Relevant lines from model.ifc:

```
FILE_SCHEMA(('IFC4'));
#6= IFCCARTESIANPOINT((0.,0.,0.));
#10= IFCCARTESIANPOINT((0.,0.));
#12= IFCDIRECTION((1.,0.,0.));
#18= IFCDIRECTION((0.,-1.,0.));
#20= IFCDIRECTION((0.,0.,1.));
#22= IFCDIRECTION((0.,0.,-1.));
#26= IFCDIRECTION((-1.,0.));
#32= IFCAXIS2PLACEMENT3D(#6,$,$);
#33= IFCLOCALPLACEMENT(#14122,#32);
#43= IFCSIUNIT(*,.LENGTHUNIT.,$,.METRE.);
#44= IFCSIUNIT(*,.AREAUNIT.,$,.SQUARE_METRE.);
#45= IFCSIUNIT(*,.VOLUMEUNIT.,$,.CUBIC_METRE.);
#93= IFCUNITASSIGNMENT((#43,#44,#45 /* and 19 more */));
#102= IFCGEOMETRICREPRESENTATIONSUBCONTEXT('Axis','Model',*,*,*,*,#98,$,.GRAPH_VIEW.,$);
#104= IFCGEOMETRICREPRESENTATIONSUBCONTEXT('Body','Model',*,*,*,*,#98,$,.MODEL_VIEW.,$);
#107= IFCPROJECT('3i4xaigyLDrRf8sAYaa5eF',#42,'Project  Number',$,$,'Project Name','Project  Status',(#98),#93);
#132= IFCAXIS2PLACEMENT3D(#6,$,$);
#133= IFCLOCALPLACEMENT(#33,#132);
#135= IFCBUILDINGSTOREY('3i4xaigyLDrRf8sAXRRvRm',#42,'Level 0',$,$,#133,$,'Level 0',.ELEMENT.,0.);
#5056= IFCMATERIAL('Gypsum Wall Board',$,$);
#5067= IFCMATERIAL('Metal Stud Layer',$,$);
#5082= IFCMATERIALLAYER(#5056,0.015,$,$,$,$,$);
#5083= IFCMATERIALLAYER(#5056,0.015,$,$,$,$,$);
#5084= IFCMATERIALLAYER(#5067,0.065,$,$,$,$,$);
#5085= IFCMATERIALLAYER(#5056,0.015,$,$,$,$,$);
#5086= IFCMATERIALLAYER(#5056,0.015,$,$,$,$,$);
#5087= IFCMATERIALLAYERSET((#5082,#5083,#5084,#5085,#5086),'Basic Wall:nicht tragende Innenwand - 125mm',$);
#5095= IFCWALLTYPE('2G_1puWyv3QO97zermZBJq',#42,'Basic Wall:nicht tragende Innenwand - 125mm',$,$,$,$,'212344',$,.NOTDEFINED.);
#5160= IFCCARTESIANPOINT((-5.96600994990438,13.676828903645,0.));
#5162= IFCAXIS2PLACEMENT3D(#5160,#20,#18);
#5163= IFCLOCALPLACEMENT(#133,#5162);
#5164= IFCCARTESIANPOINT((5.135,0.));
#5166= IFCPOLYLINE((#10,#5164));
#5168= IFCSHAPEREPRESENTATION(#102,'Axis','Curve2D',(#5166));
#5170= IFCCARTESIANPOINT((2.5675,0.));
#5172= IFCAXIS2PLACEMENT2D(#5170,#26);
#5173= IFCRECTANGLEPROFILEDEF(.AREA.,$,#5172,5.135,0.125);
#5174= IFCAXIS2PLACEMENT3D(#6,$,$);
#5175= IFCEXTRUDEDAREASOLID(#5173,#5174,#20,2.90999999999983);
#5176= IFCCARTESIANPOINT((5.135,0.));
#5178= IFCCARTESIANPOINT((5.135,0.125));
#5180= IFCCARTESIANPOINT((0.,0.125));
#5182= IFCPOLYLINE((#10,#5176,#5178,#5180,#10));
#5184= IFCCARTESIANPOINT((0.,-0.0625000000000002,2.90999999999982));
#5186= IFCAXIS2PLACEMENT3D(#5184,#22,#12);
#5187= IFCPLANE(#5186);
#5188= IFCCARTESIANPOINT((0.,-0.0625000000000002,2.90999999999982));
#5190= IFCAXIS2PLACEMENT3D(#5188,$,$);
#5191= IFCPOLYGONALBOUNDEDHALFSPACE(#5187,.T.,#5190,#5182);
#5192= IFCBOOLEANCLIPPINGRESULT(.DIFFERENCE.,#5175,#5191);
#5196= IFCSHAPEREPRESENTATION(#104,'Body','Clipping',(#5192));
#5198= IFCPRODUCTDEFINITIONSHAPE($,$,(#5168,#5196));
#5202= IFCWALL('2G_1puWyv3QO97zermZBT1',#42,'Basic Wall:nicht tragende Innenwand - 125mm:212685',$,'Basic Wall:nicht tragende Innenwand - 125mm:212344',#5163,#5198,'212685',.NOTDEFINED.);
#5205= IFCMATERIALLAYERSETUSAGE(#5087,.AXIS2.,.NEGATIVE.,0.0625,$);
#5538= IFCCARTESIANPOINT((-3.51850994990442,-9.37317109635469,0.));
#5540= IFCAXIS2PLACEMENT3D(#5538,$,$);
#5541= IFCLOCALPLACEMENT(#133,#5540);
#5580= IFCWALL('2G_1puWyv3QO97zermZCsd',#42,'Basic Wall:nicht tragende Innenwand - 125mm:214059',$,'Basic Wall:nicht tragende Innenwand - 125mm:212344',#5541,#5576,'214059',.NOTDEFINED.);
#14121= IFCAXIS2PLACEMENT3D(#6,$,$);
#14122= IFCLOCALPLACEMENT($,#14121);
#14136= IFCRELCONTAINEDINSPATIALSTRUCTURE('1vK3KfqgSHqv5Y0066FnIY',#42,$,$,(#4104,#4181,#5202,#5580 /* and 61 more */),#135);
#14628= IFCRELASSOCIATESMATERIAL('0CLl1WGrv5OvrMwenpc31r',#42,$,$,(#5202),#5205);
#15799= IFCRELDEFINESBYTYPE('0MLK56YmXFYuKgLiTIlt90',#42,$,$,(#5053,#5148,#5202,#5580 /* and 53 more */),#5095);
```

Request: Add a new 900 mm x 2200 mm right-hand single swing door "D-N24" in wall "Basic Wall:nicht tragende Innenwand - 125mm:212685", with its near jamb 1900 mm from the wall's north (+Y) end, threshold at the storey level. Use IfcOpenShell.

```python
import numpy as np
import ifcopenshell
import ifcopenshell.api.feature
import ifcopenshell.api.geometry
import ifcopenshell.api.root
import ifcopenshell.api.spatial
import ifcopenshell.geom
import ifcopenshell.util.element
import ifcopenshell.util.placement
import ifcopenshell.util.representation
import ifcopenshell.util.shape
import ifcopenshell.util.unit

model = ifcopenshell.open("model.ifc")
unit_scale = ifcopenshell.util.unit.calculate_unit_scale(model)
settings = ifcopenshell.geom.settings()


def volume(element):
    """Net volume in cubic metres, openings subtracted."""
    shape = ifcopenshell.geom.create_shape(settings, element)
    return ifcopenshell.util.shape.get_volume(shape.geometry)


wall = model.by_id(5202)
storey = ifcopenshell.util.element.get_container(wall, ifc_class="IfcBuildingStorey")
context = ifcopenshell.util.representation.get_context(model, "Model", "Body", "MODEL_VIEW")
before = volume(wall)

width, height, from_end, sill = 0.9, 2.2, 1.9, 0.0  # metres

# The wall runs along its own X axis, and the end named is its -X end.
wall_shape = ifcopenshell.geom.create_shape(settings, wall)
x, y, z = ifcopenshell.util.shape.get_vertices(wall_shape.geometry).T
start = x.min() + from_end
face, thickness = float(y.min()), float(y.max() - y.min())
wall_matrix = ifcopenshell.util.placement.get_local_placement(wall.ObjectPlacement)
level = ifcopenshell.util.placement.get_local_placement(storey.ObjectPlacement)[2, 3]


def in_wall(x, y):
    """Placement at x, y metres in the wall's axes, at sill height."""
    matrix = wall_matrix.copy()
    matrix[:, 3] = wall_matrix @ np.array([x / unit_scale, y / unit_scale, 0.0, 1.0])
    matrix[2, 3] = level + sill / unit_scale
    return matrix


# Opening: a box that overshoots both wall faces by 50 mm.
opening = ifcopenshell.api.root.create_entity(model, ifc_class="IfcOpeningElement", predefined_type="OPENING")
box = ifcopenshell.api.geometry.add_wall_representation(
    model, context=context, length=width, height=height, thickness=thickness + 0.1
)
ifcopenshell.api.geometry.assign_representation(model, product=opening, representation=box)
ifcopenshell.api.geometry.edit_object_placement(model, product=opening, matrix=in_wall(start, face - 0.05), is_si=False)
ifcopenshell.api.feature.add_feature(model, feature=opening, element=wall)

door = ifcopenshell.api.root.create_entity(model, ifc_class="IfcDoor", name="D-N24", predefined_type="DOOR")
door.OverallWidth, door.OverallHeight = width / unit_scale, height / unit_scale
door.OperationType = "SINGLE_SWING_RIGHT"
body = ifcopenshell.api.geometry.add_door_representation(
    model,
    context=context,
    overall_width=door.OverallWidth,
    overall_height=door.OverallHeight,
    operation_type="SINGLE_SWING_RIGHT",
    lining_properties={"LiningDepth": thickness / unit_scale, "ThresholdDepth": thickness / unit_scale},
)
ifcopenshell.api.geometry.assign_representation(model, product=door, representation=body)
ifcopenshell.api.spatial.assign_container(model, products=[door], relating_structure=storey)
ifcopenshell.api.feature.add_filling(model, opening=opening, element=door)

# The lining spans the wall, so the door starts at the wall face.
ifcopenshell.api.geometry.edit_object_placement(model, product=door, matrix=in_wall(start, face), is_si=False)

after = volume(wall)

print(f"wall volume {before:.3f} -> {after:.3f} m3")

model.write("model_v2.ifc")
```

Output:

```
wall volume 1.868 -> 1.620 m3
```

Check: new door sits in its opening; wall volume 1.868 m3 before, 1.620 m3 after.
